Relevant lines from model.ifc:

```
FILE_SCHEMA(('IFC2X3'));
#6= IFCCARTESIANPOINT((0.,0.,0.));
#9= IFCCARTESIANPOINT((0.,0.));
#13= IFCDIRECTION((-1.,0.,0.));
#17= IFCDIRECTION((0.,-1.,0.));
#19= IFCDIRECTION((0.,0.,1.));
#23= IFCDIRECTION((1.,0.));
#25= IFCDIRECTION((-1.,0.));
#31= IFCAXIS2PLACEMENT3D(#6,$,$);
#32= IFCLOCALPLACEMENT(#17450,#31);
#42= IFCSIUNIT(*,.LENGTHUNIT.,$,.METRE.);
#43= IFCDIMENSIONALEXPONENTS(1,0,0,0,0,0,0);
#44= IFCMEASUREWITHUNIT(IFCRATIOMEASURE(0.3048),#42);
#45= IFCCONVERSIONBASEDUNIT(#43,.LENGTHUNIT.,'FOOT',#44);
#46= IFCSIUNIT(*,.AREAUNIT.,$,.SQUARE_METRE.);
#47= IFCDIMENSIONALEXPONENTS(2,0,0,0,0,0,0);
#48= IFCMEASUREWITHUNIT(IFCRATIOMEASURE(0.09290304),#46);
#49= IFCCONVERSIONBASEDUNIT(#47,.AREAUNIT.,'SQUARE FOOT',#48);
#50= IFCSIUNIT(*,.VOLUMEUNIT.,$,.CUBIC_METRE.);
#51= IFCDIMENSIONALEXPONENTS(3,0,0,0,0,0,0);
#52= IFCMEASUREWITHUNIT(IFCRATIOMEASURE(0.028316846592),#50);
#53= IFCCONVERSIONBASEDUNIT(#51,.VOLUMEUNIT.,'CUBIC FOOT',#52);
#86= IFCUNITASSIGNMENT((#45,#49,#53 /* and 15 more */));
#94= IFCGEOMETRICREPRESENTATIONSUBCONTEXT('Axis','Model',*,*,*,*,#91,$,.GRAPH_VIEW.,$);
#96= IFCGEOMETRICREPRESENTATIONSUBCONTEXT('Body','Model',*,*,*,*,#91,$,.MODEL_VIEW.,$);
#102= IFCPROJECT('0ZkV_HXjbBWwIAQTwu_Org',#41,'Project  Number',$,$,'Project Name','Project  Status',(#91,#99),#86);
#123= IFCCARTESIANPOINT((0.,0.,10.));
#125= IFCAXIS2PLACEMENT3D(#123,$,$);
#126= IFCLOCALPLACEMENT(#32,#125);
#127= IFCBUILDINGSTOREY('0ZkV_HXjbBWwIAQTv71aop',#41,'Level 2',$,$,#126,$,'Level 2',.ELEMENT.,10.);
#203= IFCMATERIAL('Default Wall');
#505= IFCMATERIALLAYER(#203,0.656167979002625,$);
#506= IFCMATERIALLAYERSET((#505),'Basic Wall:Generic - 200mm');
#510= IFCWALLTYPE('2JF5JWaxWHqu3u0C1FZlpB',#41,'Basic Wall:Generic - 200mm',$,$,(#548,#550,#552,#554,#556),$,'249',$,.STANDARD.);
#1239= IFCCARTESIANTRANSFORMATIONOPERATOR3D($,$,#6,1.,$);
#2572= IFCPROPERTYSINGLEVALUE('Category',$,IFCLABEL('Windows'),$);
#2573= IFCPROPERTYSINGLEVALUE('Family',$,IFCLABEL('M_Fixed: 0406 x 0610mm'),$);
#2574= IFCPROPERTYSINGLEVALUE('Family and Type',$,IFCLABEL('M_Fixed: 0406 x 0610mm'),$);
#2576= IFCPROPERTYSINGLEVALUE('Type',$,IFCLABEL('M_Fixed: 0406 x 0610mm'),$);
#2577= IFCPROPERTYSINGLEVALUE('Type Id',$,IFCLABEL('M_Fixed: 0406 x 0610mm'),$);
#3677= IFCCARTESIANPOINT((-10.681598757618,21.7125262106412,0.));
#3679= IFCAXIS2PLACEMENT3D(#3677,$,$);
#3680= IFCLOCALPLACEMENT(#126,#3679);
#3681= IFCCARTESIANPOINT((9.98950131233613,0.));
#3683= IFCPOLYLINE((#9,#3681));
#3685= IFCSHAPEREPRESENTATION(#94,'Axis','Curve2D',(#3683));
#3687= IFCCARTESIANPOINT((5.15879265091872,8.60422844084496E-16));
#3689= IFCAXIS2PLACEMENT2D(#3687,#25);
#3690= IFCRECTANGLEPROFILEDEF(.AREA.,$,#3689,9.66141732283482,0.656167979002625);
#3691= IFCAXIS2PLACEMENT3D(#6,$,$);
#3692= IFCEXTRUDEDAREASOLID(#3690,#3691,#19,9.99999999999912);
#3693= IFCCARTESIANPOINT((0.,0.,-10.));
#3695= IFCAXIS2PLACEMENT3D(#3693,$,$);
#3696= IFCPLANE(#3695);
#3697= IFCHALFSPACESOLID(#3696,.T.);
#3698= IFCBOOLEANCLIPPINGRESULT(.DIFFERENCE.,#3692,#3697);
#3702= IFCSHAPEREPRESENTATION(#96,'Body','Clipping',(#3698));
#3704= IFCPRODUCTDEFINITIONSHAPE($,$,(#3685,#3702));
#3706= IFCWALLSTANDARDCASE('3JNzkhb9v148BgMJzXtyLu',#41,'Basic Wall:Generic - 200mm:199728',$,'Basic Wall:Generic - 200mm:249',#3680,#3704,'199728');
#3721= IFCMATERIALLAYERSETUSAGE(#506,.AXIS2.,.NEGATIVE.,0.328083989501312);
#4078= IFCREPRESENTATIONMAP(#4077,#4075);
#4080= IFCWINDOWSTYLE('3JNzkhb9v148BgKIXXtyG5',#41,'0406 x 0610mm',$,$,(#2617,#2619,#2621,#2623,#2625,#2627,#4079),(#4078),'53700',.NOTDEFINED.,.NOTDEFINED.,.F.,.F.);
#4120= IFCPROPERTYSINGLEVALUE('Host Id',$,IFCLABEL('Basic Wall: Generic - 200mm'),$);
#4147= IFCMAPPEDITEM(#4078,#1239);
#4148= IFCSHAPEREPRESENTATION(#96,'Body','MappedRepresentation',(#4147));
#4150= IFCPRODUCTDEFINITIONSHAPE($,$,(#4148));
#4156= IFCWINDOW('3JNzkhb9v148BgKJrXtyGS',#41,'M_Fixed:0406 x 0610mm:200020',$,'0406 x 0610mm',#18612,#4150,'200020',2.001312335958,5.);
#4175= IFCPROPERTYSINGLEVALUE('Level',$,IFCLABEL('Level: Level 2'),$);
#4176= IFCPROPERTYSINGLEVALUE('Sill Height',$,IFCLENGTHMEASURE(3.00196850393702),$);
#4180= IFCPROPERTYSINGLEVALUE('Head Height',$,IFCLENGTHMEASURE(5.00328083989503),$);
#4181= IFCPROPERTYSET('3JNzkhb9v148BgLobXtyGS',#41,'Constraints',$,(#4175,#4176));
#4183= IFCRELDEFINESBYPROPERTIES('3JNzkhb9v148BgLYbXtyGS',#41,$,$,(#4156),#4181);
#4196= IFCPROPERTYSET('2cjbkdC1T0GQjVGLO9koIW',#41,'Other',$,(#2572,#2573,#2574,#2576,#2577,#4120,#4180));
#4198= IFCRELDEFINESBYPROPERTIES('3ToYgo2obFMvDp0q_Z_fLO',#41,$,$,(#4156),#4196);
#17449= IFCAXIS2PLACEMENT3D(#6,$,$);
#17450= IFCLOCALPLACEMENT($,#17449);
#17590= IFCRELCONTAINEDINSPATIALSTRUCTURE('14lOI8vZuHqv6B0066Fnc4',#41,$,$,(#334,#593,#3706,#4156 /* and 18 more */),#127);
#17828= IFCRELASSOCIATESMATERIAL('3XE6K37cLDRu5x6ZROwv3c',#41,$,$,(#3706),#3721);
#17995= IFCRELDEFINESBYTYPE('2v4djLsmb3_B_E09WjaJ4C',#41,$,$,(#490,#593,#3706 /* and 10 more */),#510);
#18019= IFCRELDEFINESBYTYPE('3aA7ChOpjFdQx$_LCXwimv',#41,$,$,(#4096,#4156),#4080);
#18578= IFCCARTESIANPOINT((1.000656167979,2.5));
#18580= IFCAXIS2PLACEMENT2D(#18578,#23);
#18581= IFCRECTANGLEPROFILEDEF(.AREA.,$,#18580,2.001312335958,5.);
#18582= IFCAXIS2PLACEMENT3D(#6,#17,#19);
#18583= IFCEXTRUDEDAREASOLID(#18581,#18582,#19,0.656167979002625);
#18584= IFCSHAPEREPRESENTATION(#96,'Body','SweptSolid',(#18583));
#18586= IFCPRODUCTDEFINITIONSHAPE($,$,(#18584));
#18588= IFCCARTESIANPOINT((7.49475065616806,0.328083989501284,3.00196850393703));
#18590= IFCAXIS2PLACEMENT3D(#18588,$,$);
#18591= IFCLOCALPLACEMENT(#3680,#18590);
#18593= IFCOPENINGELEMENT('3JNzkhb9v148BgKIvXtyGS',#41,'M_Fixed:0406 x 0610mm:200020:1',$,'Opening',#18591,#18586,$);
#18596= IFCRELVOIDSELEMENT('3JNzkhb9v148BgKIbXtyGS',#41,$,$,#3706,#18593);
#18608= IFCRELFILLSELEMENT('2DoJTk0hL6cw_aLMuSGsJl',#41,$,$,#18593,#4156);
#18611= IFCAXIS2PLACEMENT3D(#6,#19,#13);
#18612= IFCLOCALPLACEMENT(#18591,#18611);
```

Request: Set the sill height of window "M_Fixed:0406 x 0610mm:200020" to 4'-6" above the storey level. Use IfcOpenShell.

```python
import numpy as np
import ifcopenshell
import ifcopenshell.api.geometry
import ifcopenshell.api.pset
import ifcopenshell.geom
import ifcopenshell.util.element
import ifcopenshell.util.placement
import ifcopenshell.util.shape
import ifcopenshell.util.unit

model = ifcopenshell.open("model.ifc")
unit_scale = ifcopenshell.util.unit.calculate_unit_scale(model)

window = model.by_guid("3JNzkhb9v148BgKJrXtyGS")
opening = window.FillsVoids[0].RelatingOpeningElement
storey = ifcopenshell.util.element.get_container(window, ifc_class="IfcBuildingStorey")
level = ifcopenshell.util.placement.get_local_placement(storey.ObjectPlacement)[2, 3]

# The opening's origin need not be at the sill, so measure its lowest point.
shape = ifcopenshell.geom.create_shape(ifcopenshell.geom.settings(), opening)
bottom = ifcopenshell.util.shape.get_shape_bottom_elevation(shape, shape.geometry) / unit_scale
dz = level + 54 * 0.0254 / unit_scale - bottom

shift = np.array([0.0, 0.0, dz])
# The window is placed relative to its opening, so it follows when the opening moves.
matrix = ifcopenshell.util.placement.get_local_placement(opening.ObjectPlacement)
matrix[:3, 3] += shift
ifcopenshell.api.geometry.edit_object_placement(
    model, product=opening, matrix=matrix, is_si=False, should_transform_children=True
)

# Keep the stored heights in step.
pset = model.by_id(ifcopenshell.util.element.get_pset(window, "Constraints", should_inherit=False)["id"])
ifcopenshell.api.pset.edit_pset(model, pset=pset, properties={
    "Sill Height": model.create_entity("IfcLengthMeasure", ifcopenshell.util.element.get_pset(window, "Constraints", "Sill Height") + dz),
})
pset = model.by_id(ifcopenshell.util.element.get_pset(window, "Other", should_inherit=False)["id"])
ifcopenshell.api.pset.edit_pset(model, pset=pset, properties={
    "Head Height": model.create_entity("IfcLengthMeasure", ifcopenshell.util.element.get_pset(window, "Other", "Head Height") + dz),
})

print(f"moved by {dz * unit_scale:+.3f} m")

model.write("model-out.ifc")
```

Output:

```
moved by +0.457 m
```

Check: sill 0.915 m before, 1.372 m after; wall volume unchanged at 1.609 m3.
